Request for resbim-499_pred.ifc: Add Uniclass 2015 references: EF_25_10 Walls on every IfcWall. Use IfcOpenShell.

First a look at what the model holds.

```python
import ifcopenshell

model = ifcopenshell.open("resbim-499_pred.ifc")
print(model.schema)
print("classifications:", [c.Name for c in model.by_type("IfcClassification")])
for ifc_class in ("IfcDoor", "IfcRoof", "IfcStair", "IfcWall", "IfcWindow"):
    print(ifc_class, len(model.by_type(ifc_class)))
```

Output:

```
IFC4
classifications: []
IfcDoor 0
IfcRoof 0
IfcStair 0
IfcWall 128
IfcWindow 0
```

```python
import ifcopenshell
import ifcopenshell.api.classification

model = ifcopenshell.open("resbim-499_pred.ifc")

system = ifcopenshell.api.classification.add_classification(model, classification="Uniclass 2015")

codes = {
    "IfcWall": ("EF_25_10", "Walls"),
}
for ifc_class, (code, name) in codes.items():
    products = model.by_type(ifc_class)
    ifcopenshell.api.classification.add_reference(
        model, products=products, classification=system, identification=code, name=name
    )
    print(code, len(products))

model.write("resbim-499_pred-out.ifc")
```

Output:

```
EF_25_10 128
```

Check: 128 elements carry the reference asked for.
